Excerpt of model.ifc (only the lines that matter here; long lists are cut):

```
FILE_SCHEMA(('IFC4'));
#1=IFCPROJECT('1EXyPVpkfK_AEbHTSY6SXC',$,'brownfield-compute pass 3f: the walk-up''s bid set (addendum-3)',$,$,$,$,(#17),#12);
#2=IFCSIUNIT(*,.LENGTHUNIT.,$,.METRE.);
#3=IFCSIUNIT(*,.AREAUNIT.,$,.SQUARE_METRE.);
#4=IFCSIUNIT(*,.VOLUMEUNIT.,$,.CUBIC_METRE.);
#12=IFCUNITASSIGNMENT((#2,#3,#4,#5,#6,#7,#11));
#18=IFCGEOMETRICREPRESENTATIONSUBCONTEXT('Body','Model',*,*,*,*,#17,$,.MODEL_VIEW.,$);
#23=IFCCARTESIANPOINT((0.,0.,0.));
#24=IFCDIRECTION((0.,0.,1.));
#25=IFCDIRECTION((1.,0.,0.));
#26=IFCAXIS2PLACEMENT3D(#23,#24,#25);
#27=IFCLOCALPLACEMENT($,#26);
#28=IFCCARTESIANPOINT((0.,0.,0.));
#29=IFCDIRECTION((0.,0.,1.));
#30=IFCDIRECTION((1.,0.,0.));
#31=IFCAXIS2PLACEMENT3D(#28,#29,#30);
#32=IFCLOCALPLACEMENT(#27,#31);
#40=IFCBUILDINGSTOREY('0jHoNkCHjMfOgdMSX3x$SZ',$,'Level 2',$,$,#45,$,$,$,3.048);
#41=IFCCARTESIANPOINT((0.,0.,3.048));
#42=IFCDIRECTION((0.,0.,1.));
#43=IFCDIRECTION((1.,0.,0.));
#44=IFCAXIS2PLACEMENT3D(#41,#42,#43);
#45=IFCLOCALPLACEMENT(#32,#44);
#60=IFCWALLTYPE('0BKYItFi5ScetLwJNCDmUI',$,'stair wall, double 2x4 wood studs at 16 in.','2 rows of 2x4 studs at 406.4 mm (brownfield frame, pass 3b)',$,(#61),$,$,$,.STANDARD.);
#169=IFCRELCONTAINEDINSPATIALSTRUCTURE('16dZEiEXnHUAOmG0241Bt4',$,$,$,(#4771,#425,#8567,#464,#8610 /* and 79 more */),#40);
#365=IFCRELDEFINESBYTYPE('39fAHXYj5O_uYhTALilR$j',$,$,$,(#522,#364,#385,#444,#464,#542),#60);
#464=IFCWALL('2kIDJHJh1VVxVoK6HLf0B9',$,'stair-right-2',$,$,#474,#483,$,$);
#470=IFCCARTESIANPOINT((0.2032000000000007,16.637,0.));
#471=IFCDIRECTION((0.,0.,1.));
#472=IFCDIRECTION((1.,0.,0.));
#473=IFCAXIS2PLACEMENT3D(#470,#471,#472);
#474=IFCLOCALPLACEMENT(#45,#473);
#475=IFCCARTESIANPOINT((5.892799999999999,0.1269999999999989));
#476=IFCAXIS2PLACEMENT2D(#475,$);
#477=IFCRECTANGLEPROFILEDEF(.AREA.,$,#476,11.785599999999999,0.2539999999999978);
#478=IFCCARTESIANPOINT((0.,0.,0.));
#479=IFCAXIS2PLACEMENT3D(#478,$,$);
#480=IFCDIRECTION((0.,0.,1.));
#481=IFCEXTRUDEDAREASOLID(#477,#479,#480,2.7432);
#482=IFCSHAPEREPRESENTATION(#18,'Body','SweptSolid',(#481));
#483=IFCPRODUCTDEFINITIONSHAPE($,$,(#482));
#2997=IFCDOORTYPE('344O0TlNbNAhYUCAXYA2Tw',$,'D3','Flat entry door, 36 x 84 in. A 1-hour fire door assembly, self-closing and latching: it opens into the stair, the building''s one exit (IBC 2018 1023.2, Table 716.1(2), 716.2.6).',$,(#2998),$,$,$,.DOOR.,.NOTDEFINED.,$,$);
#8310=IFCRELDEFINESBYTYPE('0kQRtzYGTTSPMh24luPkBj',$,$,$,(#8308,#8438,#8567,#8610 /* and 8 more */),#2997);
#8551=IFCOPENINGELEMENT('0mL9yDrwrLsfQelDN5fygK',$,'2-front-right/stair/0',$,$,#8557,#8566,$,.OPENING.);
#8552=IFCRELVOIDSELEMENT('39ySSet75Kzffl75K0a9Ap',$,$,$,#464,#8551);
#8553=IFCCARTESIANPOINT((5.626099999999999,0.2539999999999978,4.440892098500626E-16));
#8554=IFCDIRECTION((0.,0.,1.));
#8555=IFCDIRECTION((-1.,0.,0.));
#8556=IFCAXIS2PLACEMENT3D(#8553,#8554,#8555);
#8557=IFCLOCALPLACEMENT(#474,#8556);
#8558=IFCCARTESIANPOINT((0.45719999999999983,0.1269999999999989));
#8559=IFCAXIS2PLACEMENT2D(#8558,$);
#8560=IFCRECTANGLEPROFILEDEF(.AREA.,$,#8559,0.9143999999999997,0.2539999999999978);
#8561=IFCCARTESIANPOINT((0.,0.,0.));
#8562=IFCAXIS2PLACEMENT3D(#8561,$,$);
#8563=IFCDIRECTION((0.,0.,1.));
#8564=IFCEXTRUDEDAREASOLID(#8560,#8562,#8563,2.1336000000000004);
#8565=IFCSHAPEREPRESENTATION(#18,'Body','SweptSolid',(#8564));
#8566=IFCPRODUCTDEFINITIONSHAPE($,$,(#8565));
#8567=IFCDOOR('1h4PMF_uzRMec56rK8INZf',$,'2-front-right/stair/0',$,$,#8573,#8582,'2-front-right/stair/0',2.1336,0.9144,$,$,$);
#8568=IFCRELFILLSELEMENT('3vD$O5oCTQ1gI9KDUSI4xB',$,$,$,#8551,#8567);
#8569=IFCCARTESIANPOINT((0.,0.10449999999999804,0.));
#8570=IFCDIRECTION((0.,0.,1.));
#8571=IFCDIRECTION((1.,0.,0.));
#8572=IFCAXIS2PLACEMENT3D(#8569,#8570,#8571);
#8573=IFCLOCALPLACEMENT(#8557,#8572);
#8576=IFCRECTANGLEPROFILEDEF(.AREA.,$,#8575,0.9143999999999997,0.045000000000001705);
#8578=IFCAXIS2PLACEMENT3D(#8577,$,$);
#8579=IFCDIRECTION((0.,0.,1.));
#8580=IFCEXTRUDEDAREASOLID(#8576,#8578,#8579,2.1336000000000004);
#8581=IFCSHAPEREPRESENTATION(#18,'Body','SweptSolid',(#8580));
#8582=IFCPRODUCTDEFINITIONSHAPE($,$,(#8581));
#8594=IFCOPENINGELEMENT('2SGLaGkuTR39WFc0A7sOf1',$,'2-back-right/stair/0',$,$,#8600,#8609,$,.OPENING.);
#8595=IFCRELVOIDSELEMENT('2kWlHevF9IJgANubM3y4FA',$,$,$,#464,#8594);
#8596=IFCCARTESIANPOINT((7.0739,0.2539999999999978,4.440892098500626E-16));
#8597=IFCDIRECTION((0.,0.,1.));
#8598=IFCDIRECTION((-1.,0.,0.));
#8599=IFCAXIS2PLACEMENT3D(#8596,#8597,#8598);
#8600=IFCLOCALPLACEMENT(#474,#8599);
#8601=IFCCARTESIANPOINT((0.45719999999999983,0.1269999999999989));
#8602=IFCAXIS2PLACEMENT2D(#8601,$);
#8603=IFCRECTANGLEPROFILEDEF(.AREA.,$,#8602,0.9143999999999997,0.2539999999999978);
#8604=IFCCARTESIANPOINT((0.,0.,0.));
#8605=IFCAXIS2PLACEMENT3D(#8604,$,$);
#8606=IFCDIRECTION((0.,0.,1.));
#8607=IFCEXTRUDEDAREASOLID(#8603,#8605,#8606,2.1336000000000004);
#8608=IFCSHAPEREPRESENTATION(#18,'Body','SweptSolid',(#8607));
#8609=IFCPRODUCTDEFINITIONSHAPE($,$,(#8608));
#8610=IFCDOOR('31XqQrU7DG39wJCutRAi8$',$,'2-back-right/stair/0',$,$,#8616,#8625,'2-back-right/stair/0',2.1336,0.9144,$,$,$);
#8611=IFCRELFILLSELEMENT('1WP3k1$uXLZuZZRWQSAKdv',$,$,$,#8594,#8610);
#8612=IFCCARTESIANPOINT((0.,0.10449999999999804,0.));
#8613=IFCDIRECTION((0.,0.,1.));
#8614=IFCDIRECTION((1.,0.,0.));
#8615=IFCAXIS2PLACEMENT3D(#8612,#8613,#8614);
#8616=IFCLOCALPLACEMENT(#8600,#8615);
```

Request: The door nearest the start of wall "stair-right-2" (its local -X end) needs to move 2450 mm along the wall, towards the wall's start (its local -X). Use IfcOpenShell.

```python
import ifcopenshell
import ifcopenshell.api.geometry
import ifcopenshell.util.placement
import ifcopenshell.util.unit

model = ifcopenshell.open("model.ifc")
unit_scale = ifcopenshell.util.unit.calculate_unit_scale(model)

door = model.by_guid("1h4PMF_uzRMec56rK8INZf")
opening = door.FillsVoids[0].RelatingOpeningElement
wall = opening.VoidsElements[0].RelatingBuildingElement

wall_matrix = ifcopenshell.util.placement.get_local_placement(wall.ObjectPlacement)
shift = wall_matrix[:3, 0] * -2.45 / unit_scale
before = ifcopenshell.util.placement.get_local_placement(door.ObjectPlacement)[:3, 3].copy()

# The door is placed relative to its opening, so it follows when the opening moves.
matrix = ifcopenshell.util.placement.get_local_placement(opening.ObjectPlacement)
matrix[:3, 3] += shift
ifcopenshell.api.geometry.edit_object_placement(
    model, product=opening, matrix=matrix, is_si=False, should_transform_children=True
)

after = ifcopenshell.util.placement.get_local_placement(door.ObjectPlacement)[:3, 3]
print("door moved by", (after - before).round(3) + 0.0)

model.write("model_edited.ifc")
```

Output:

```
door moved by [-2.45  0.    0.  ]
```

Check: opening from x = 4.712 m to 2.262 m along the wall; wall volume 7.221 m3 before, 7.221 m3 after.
